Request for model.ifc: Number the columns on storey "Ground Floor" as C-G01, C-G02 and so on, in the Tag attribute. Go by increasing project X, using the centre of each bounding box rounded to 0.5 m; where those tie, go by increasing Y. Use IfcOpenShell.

First a look at what the model holds.

```python
import ifcopenshell
import ifcopenshell.util.element
import ifcopenshell.util.placement

model = ifcopenshell.open("model.ifc")
print(model.schema)
storey = next(s for s in model.by_type("IfcBuildingStorey") if s.Name == "Ground Floor")
columns = [e for e in ifcopenshell.util.element.get_decomposition(storey) if e.is_a("IfcColumn")]
for e in sorted(columns, key=lambda e: e.id()):
    origin = ifcopenshell.util.placement.get_local_placement(e.ObjectPlacement)[:3, 3]
    print(e.id(), e.Tag, e.Name, origin.round(2) + 0.0, sep=" | ")
```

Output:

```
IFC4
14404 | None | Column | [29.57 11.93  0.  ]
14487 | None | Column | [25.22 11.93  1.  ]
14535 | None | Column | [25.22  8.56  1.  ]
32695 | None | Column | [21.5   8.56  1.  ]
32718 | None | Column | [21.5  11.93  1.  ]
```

```python
import ifcopenshell
import ifcopenshell.geom
import ifcopenshell.util.element
import ifcopenshell.util.shape

model = ifcopenshell.open("model.ifc")
settings = ifcopenshell.geom.settings()
settings.set("use-world-coords", True)


def centre(element):
    shape = ifcopenshell.geom.create_shape(settings, element)
    return ifcopenshell.util.shape.get_bbox_centroid(shape.geometry)


storey = next(s for s in model.by_type("IfcBuildingStorey") if s.Name == "Ground Floor")
columns = [e for e in ifcopenshell.util.element.get_decomposition(storey) if e.is_a("IfcColumn")]

# Insertion points can sit at a corner or the storey origin, so sort by the geometry (in metres).
centres = {e: centre(e) for e in columns}
columns.sort(key=lambda e: (round(centres[e][0] / 0.5), centres[e][1]))

for i, e in enumerate(columns, start=1):
    number = f"C-G{i:02d}"
    e.Tag = number
    print(e.id(), number)

model.write("model-out.ifc")
```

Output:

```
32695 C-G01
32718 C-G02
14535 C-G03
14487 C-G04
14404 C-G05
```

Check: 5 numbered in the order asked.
